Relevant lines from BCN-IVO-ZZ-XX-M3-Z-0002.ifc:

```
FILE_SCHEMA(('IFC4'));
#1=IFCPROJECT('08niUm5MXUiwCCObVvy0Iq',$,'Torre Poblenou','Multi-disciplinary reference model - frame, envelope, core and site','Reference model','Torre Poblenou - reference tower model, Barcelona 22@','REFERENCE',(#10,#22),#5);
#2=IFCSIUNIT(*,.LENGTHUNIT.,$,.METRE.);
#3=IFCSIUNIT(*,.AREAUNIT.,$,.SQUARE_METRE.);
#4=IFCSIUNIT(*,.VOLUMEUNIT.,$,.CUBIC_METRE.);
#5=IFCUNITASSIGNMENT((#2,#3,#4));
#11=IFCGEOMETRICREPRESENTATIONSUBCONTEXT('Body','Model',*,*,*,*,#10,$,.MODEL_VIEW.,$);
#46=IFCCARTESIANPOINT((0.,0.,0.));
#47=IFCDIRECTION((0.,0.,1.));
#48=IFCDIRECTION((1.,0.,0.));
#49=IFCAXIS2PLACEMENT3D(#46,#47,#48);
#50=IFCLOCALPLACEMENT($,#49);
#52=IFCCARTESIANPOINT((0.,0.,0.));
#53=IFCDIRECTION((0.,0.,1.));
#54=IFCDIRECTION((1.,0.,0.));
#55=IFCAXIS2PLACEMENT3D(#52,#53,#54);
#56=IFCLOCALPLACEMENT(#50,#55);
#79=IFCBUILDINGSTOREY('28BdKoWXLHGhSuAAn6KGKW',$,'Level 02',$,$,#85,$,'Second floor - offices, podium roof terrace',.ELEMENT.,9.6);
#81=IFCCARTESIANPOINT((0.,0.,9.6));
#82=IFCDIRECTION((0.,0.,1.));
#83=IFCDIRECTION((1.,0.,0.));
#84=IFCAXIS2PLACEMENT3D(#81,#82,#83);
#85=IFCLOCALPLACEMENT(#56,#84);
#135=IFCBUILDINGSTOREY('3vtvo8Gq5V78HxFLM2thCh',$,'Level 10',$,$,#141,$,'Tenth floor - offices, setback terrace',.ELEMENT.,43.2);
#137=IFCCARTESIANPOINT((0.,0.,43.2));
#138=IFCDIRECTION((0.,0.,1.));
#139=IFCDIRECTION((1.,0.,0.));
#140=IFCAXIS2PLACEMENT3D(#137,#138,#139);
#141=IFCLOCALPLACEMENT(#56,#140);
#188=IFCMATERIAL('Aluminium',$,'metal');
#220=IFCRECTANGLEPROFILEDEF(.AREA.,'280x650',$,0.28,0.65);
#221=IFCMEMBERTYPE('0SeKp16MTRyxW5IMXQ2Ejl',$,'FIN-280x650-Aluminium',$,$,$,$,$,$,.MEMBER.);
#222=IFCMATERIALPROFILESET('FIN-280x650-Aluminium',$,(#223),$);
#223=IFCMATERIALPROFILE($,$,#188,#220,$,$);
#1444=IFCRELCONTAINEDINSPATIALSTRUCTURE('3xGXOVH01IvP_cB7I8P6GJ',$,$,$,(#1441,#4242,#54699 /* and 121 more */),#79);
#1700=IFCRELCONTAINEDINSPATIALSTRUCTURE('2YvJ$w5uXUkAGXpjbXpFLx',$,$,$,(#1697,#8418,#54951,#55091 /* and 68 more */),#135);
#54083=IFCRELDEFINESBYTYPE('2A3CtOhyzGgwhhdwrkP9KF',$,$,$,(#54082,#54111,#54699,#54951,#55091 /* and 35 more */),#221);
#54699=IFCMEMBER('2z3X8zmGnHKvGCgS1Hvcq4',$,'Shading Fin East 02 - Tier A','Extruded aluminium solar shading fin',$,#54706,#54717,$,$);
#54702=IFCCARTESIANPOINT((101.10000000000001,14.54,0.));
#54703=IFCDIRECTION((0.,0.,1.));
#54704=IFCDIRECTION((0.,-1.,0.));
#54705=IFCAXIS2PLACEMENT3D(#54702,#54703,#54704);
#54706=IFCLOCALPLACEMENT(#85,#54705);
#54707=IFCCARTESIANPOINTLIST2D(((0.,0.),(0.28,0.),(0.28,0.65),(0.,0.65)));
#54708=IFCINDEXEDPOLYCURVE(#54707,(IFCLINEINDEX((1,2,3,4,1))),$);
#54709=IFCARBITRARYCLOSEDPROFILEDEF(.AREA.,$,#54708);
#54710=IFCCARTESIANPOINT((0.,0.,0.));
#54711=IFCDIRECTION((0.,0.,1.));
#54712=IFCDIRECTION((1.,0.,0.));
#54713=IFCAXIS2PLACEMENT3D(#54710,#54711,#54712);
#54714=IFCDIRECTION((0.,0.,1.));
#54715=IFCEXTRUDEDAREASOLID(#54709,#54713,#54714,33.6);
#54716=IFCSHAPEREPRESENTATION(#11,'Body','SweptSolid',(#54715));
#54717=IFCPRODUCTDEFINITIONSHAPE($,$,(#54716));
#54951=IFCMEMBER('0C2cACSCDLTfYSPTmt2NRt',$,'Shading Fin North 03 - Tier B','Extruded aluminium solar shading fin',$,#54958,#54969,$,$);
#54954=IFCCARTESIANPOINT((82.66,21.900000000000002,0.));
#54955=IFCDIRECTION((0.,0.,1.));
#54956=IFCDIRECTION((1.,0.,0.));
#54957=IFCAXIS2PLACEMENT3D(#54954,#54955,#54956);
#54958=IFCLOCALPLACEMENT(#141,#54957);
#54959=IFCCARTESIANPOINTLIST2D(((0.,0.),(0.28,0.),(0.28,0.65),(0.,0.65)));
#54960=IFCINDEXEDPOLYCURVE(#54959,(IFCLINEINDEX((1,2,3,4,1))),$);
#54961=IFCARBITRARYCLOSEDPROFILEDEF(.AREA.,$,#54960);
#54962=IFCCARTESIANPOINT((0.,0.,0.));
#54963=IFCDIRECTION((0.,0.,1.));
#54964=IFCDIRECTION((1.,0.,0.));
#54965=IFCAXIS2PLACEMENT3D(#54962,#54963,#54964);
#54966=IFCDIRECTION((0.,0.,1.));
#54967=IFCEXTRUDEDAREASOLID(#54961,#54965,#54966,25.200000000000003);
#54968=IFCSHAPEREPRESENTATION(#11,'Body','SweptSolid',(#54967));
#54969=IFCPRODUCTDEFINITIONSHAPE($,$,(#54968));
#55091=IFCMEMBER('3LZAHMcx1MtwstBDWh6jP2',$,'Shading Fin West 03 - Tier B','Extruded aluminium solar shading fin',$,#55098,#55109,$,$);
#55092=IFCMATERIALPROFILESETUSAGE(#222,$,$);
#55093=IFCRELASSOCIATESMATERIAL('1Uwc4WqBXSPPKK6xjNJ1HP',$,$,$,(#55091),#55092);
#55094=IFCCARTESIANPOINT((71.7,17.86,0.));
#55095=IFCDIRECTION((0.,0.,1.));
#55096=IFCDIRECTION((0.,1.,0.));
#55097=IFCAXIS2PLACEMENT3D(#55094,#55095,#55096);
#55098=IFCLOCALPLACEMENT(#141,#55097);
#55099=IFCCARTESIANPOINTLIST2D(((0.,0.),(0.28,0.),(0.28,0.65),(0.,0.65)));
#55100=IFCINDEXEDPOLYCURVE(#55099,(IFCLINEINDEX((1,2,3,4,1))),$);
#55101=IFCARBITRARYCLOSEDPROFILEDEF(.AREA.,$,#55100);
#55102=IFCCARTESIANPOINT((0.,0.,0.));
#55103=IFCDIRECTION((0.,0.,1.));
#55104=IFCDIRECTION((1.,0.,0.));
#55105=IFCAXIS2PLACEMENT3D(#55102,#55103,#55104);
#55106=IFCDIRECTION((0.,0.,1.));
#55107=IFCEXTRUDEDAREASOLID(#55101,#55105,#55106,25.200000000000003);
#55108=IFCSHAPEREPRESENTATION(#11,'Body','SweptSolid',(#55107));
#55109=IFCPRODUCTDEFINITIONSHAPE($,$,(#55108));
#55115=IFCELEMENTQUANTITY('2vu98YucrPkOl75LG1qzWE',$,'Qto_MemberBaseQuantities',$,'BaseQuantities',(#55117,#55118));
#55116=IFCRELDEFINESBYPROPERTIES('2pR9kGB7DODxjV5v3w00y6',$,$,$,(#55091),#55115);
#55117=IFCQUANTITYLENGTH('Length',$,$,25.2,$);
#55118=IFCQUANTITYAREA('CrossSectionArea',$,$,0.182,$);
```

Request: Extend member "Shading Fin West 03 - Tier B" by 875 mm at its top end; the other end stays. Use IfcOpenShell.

```python
import ifcopenshell
import ifcopenshell.api.pset
import ifcopenshell.util.element
import ifcopenshell.util.representation
import ifcopenshell.util.unit

model = ifcopenshell.open("BCN-IVO-ZZ-XX-M3-Z-0002.ifc")
unit_scale = ifcopenshell.util.unit.calculate_unit_scale(model)

member = model.by_guid("3LZAHMcx1MtwstBDWh6jP2")
change = 0.875 / unit_scale

# The extrusion runs towards the end named, so only its depth changes.
body = ifcopenshell.util.representation.get_representation(member, "Model", "Body")
solid = body.Items[0]
old_length = solid.Depth
solid.Depth += change

# Update the stored length and volume.
qto = model.by_id(ifcopenshell.util.element.get_pset(member, "Qto_MemberBaseQuantities", should_inherit=False)["id"])
ifcopenshell.api.pset.edit_qto(model, qto=qto, properties={"Length": solid.Depth})

print(f"length {old_length:g} -> {solid.Depth:g}")

model.write("BCN-IVO-ZZ-XX-M3-Z-0002_v2.ifc")
```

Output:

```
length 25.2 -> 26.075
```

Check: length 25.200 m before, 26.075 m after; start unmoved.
